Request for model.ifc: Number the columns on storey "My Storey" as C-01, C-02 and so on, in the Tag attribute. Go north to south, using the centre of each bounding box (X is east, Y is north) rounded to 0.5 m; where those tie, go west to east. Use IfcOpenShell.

First a look at what the model holds.

```python
import ifcopenshell
import ifcopenshell.util.element
import ifcopenshell.util.placement

model = ifcopenshell.open("model.ifc")
print(model.schema)
storey = next(s for s in model.by_type("IfcBuildingStorey") if s.Name == "My Storey")
columns = [e for e in ifcopenshell.util.element.get_decomposition(storey) if e.is_a("IfcColumn")]
for e in sorted(columns, key=lambda e: e.id()):
    origin = ifcopenshell.util.placement.get_local_placement(e.ObjectPlacement)[:3, 3]
    print(e.id(), e.Tag, e.Name, origin.round(2) + 0.0, sep=" | ")
```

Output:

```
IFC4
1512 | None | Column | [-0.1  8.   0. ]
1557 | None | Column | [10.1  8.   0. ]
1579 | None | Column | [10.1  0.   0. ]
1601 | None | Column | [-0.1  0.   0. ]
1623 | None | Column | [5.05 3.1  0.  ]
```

```python
import ifcopenshell
import ifcopenshell.geom
import ifcopenshell.util.element
import ifcopenshell.util.shape

model = ifcopenshell.open("model.ifc")
settings = ifcopenshell.geom.settings()
settings.set("use-world-coords", True)


def centre(element):
    shape = ifcopenshell.geom.create_shape(settings, element)
    return ifcopenshell.util.shape.get_bbox_centroid(shape.geometry)


storey = next(s for s in model.by_type("IfcBuildingStorey") if s.Name == "My Storey")
columns = [e for e in ifcopenshell.util.element.get_decomposition(storey) if e.is_a("IfcColumn")]

# Insertion points can sit at a corner or the storey origin, so sort by the geometry (in metres).
centres = {e: centre(e) for e in columns}
columns.sort(key=lambda e: (-round(centres[e][1] / 0.5), centres[e][0]))

for i, e in enumerate(columns, start=1):
    number = f"C-{i:02d}"
    e.Tag = number
    print(e.id(), number)

model.write("model_updated.ifc")
```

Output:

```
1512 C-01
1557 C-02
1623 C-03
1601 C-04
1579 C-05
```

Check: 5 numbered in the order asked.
